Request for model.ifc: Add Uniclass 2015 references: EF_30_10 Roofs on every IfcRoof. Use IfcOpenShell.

First a look at what the model holds.

```python
import ifcopenshell

model = ifcopenshell.open("model.ifc")
print(model.schema)
print("classifications:", [c.Name for c in model.by_type("IfcClassification")])
for ifc_class in ("IfcDoor", "IfcRoof", "IfcStair", "IfcWall", "IfcWindow"):
    print(ifc_class, len(model.by_type(ifc_class)))
```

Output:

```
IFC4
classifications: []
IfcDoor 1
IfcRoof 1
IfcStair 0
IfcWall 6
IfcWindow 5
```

```python
import ifcopenshell
import ifcopenshell.api.classification

model = ifcopenshell.open("model.ifc")

system = ifcopenshell.api.classification.add_classification(model, classification="Uniclass 2015")

codes = {
    "IfcRoof": ("EF_30_10", "Roofs"),
}
for ifc_class, (code, name) in codes.items():
    products = model.by_type(ifc_class)
    ifcopenshell.api.classification.add_reference(
        model, products=products, classification=system, identification=code, name=name
    )
    print(code, len(products))

model.write("model_edited.ifc")
```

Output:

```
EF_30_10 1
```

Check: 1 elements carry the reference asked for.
